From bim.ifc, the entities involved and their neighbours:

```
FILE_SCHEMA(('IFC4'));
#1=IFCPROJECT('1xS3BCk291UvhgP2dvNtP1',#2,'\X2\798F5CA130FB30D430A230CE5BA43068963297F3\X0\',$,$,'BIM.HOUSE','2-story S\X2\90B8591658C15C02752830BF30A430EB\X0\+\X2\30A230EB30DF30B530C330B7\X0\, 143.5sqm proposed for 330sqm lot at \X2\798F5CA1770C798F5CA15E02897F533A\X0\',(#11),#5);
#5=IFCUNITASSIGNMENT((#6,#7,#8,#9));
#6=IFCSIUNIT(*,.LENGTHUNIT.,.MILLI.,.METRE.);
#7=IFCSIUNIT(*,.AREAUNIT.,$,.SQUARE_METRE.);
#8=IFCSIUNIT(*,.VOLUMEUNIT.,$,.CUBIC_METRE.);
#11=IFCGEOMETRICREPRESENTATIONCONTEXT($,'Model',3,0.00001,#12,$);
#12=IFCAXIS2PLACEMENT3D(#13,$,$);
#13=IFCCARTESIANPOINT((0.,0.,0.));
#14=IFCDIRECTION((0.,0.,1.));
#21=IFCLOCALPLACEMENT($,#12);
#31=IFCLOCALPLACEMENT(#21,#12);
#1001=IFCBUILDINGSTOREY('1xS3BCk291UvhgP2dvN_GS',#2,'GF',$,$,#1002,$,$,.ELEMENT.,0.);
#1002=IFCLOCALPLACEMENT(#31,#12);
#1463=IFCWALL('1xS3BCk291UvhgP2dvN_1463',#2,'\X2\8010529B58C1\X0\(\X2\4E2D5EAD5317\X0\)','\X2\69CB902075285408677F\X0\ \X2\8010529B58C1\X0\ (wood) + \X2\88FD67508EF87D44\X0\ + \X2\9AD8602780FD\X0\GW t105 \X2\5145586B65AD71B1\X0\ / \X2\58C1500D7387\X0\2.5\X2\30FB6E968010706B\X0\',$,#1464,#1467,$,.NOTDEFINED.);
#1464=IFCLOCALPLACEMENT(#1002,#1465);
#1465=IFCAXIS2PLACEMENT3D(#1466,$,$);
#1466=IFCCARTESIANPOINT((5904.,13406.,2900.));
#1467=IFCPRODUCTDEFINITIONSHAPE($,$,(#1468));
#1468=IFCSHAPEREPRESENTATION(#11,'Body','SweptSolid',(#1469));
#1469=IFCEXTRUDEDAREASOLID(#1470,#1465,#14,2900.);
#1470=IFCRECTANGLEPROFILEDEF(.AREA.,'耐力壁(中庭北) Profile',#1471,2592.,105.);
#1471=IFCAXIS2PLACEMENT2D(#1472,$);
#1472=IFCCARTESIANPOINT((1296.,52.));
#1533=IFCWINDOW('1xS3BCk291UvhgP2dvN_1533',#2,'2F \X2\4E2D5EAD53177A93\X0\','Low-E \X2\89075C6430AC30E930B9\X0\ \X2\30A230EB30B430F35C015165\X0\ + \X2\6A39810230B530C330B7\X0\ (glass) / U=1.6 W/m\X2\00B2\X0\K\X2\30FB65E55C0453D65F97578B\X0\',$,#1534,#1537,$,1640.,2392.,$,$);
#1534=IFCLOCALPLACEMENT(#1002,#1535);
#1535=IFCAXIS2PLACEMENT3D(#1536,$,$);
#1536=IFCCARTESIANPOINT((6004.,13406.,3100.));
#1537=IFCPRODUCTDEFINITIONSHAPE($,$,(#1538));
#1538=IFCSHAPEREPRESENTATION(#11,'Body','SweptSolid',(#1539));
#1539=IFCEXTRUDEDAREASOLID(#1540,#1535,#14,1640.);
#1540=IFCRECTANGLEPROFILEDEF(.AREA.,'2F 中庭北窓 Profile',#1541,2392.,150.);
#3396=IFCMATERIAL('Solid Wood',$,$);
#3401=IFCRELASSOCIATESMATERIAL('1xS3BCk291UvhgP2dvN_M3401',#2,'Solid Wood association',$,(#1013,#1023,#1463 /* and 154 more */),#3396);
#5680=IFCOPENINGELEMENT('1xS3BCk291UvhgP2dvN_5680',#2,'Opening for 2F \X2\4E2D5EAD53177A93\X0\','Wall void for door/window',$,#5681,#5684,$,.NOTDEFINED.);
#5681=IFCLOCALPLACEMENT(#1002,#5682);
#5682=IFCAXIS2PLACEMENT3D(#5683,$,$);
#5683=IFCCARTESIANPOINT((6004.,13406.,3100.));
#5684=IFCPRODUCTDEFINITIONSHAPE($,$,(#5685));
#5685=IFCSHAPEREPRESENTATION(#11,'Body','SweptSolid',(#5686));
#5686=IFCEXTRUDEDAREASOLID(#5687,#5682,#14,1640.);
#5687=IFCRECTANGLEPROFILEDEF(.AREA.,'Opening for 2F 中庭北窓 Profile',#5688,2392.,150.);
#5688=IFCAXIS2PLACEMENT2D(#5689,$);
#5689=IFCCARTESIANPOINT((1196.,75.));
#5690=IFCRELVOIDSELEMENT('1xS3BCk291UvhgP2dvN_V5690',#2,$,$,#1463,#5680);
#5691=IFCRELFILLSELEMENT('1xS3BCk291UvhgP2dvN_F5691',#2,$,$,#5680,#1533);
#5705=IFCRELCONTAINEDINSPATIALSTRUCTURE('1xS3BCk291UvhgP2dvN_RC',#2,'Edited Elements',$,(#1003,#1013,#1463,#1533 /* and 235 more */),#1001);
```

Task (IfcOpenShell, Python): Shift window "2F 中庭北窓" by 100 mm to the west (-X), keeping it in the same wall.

```python
import ifcopenshell
import ifcopenshell.api.geometry
import ifcopenshell.util.placement

model = ifcopenshell.open("bim.ifc")

window = model.by_guid("1xS3BCk291UvhgP2dvN_1533")
opening = window.FillsVoids[0].RelatingOpeningElement
wall = opening.VoidsElements[0].RelatingBuildingElement

wall_matrix = ifcopenshell.util.placement.get_local_placement(wall.ObjectPlacement)
shift = wall_matrix[:3, 0] * -100.0
before = ifcopenshell.util.placement.get_local_placement(window.ObjectPlacement)[:3, 3].copy()

# The window is not placed relative to its opening, so move both.
for product in (opening, window):
    matrix = ifcopenshell.util.placement.get_local_placement(product.ObjectPlacement)
    matrix[:3, 3] += shift
    ifcopenshell.api.geometry.edit_object_placement(model, product=product, matrix=matrix, is_si=False)

after = ifcopenshell.util.placement.get_local_placement(window.ObjectPlacement)[:3, 3]
print("window moved by", (after - before).round(3) + 0.0)

model.write("bim_edited.ifc")
```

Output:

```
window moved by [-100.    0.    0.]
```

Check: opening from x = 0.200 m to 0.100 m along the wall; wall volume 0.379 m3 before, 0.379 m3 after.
